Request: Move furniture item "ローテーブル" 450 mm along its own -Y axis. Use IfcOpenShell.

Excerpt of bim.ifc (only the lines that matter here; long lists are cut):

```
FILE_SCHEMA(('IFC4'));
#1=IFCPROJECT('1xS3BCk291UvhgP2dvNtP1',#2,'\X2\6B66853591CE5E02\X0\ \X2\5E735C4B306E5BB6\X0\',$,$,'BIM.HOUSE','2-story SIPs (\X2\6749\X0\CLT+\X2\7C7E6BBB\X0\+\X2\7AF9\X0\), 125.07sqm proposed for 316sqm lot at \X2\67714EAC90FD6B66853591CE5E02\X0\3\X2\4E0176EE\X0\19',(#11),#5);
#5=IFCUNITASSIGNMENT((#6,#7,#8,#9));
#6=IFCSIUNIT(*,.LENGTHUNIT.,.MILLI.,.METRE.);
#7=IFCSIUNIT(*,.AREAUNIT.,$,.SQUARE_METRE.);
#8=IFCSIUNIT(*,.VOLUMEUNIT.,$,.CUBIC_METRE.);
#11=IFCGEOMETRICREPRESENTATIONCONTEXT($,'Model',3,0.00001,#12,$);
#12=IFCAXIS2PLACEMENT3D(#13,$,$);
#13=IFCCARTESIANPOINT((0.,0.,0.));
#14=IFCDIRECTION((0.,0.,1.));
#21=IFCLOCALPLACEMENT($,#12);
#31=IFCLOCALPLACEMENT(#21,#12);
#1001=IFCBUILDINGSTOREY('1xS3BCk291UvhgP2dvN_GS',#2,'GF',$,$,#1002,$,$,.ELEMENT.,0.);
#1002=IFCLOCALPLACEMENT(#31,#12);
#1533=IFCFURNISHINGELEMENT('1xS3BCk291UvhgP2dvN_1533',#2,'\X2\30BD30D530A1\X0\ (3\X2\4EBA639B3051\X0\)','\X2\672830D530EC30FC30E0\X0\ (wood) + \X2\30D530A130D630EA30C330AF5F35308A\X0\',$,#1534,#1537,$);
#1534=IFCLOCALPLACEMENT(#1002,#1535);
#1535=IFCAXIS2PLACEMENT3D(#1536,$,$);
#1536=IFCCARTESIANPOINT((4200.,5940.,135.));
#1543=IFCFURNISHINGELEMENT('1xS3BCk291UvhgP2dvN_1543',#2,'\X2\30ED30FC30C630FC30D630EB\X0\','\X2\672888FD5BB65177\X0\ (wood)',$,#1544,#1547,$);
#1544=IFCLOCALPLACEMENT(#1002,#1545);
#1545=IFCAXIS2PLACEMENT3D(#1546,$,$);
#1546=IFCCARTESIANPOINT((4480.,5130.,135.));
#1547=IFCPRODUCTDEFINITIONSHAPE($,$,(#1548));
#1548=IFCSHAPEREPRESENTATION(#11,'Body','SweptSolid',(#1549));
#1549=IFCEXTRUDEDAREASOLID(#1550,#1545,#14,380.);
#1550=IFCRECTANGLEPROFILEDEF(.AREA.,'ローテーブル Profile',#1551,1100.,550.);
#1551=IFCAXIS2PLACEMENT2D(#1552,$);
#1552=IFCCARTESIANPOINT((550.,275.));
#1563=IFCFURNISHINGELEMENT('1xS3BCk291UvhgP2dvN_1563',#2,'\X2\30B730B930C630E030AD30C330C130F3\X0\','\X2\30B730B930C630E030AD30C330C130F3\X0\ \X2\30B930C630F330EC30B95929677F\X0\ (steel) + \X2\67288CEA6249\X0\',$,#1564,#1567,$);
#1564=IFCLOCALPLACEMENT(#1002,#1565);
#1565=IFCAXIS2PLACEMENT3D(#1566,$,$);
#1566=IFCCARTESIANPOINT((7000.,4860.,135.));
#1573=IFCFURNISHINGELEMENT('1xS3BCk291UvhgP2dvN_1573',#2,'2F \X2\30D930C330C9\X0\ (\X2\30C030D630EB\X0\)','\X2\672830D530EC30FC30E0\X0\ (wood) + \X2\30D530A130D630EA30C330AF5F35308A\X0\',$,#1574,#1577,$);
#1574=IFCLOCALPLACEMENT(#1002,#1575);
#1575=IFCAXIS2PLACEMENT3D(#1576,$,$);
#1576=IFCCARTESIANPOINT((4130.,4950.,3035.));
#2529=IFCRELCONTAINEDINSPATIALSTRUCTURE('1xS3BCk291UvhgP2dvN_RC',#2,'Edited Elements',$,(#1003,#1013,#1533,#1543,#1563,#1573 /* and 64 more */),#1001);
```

```python
import ifcopenshell
import ifcopenshell.api.geometry
import ifcopenshell.util.placement

model = ifcopenshell.open("bim.ifc")

item = model.by_guid("1xS3BCk291UvhgP2dvN_1543")
matrix = ifcopenshell.util.placement.get_local_placement(item.ObjectPlacement)
matrix[:3, 3] -= matrix[:3, 1] * 450.0
ifcopenshell.api.geometry.edit_object_placement(model, product=item, matrix=matrix, is_si=False)

print(ifcopenshell.util.placement.get_local_placement(item.ObjectPlacement).round(3) + 0.0)

model.write("bim-out.ifc")
```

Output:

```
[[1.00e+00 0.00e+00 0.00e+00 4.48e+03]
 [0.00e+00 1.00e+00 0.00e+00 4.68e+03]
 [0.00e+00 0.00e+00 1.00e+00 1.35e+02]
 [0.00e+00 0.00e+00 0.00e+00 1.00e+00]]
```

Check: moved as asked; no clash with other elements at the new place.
